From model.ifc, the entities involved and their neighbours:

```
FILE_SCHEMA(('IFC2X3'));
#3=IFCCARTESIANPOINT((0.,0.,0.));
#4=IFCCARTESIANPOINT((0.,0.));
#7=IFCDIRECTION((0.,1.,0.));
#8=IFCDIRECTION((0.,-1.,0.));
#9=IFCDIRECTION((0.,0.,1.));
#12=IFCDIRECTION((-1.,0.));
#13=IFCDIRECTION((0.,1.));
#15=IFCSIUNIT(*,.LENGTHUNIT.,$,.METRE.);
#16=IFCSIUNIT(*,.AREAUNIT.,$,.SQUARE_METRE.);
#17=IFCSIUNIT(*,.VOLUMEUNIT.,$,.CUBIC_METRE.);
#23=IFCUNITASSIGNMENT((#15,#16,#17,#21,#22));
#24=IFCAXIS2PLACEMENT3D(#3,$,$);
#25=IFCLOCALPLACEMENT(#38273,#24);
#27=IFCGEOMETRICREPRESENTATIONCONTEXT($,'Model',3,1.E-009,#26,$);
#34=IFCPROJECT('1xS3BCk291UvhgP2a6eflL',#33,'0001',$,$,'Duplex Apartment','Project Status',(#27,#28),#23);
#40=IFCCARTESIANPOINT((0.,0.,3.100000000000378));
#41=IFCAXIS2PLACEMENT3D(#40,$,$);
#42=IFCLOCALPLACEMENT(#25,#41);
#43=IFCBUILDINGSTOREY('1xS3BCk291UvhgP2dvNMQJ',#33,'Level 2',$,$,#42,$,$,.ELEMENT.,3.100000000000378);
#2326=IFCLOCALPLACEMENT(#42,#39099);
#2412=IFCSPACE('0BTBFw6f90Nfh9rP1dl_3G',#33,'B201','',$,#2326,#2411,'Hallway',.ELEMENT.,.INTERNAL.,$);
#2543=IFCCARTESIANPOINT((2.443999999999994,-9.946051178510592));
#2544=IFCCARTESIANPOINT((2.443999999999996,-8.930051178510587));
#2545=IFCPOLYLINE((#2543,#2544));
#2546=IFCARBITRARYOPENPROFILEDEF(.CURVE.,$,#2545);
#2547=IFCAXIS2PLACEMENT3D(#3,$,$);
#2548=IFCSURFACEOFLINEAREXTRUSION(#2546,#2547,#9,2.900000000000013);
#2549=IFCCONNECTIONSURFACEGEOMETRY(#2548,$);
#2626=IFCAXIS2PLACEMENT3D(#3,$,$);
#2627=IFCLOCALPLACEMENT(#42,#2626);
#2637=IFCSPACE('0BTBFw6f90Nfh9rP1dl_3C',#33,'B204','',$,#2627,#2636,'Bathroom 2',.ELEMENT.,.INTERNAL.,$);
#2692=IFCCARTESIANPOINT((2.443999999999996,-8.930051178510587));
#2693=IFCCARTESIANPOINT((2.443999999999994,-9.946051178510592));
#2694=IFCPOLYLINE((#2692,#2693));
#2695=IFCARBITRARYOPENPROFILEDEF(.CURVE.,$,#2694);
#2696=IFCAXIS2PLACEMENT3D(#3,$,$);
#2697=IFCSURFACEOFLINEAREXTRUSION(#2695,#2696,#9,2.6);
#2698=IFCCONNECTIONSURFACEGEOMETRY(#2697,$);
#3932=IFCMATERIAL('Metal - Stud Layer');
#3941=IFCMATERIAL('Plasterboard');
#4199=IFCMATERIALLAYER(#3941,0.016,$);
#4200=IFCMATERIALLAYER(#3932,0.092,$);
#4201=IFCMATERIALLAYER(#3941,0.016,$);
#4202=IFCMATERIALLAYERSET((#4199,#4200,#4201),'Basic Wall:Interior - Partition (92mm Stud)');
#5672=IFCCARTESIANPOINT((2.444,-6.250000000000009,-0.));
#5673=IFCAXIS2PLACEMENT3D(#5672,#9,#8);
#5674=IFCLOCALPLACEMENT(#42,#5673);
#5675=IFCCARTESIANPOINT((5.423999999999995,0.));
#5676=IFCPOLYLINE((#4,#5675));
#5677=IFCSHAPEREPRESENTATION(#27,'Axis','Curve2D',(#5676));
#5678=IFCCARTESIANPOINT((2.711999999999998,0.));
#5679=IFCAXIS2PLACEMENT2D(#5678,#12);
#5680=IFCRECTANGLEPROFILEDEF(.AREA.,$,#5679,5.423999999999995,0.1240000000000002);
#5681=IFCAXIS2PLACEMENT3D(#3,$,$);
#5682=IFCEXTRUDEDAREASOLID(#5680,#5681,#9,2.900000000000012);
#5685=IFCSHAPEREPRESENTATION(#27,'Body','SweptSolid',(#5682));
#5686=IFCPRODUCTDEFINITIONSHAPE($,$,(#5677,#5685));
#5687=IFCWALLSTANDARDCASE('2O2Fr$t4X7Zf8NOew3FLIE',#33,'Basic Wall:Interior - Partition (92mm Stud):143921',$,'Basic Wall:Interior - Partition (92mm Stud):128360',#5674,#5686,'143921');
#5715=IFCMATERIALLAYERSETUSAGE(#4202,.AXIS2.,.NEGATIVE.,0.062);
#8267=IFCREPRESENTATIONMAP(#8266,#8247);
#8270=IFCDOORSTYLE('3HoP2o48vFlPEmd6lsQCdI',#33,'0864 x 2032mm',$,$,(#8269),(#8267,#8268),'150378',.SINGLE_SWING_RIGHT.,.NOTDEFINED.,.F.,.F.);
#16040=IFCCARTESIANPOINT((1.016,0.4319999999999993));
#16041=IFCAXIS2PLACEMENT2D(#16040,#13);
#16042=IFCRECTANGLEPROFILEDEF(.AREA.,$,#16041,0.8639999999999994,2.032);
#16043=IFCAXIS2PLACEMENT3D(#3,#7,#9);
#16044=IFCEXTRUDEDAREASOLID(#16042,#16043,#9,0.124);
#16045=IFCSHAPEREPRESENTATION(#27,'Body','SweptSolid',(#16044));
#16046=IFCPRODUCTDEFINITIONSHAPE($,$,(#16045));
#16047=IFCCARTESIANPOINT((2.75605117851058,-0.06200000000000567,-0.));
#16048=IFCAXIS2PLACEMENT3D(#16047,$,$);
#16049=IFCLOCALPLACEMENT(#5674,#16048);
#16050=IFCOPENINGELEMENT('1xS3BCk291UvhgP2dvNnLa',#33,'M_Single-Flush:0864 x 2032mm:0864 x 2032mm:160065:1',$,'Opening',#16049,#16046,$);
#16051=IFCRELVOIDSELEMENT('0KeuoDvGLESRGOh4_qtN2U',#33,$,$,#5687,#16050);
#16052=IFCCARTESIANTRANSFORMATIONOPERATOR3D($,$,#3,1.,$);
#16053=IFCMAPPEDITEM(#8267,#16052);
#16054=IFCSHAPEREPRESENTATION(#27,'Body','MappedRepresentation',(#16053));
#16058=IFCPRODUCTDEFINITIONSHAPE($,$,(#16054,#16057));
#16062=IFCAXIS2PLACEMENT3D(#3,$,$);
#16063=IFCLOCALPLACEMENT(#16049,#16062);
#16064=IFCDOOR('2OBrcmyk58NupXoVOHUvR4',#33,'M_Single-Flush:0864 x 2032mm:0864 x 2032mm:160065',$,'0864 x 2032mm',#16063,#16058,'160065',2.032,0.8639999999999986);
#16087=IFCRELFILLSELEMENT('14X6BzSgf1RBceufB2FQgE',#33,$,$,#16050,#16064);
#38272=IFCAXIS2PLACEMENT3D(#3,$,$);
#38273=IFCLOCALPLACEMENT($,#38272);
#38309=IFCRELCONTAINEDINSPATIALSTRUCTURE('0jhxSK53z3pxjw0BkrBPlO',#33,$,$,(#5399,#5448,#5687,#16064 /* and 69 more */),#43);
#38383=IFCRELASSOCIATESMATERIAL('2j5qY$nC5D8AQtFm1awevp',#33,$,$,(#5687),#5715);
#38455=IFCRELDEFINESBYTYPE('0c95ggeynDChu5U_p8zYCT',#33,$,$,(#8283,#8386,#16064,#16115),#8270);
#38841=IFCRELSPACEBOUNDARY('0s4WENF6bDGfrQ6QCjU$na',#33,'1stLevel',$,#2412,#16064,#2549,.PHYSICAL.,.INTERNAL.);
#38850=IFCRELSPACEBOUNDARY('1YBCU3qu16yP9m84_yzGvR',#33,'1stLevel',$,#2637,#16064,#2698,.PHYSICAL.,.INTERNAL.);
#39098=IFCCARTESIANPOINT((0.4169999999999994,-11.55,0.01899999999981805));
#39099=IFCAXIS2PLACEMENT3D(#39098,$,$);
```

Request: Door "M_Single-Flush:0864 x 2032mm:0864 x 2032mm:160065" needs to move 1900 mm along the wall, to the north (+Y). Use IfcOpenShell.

```python
import numpy as np
import ifcopenshell
import ifcopenshell.api.geometry
import ifcopenshell.util.placement
import ifcopenshell.util.unit

model = ifcopenshell.open("model.ifc")
unit_scale = ifcopenshell.util.unit.calculate_unit_scale(model)

door = model.by_id(16064)
opening = door.FillsVoids[0].RelatingOpeningElement
wall = opening.VoidsElements[0].RelatingBuildingElement

wall_matrix = ifcopenshell.util.placement.get_local_placement(wall.ObjectPlacement)
shift = wall_matrix[:3, 0] * -1.9 / unit_scale
before = ifcopenshell.util.placement.get_local_placement(door.ObjectPlacement)[:3, 3].copy()

# The door is placed relative to its opening, so it follows when the opening moves.
matrix = ifcopenshell.util.placement.get_local_placement(opening.ObjectPlacement)
matrix[:3, 3] += shift
ifcopenshell.api.geometry.edit_object_placement(
    model, product=opening, matrix=matrix, is_si=False, should_transform_children=True
)

# Space boundary surfaces are stored in each space's coordinates; move them too.
for rel in door.ProvidesBoundaries:
    if not rel.ConnectionGeometry:
        continue
    surface = rel.ConnectionGeometry.SurfaceOnRelatingElement
    space_matrix = ifcopenshell.util.placement.get_local_placement(rel.RelatingSpace.ObjectPlacement)
    point = np.array(surface.Position.Location.Coordinates) + space_matrix[:3, :3].T @ shift
    surface.Position = model.createIfcAxis2Placement3D(
        model.createIfcCartesianPoint(point.tolist()), surface.Position.Axis, surface.Position.RefDirection
    )

after = ifcopenshell.util.placement.get_local_placement(door.ObjectPlacement)[:3, 3]
print("door moved by", (after - before).round(3) + 0.0)

model.write("model_rev.ifc")
```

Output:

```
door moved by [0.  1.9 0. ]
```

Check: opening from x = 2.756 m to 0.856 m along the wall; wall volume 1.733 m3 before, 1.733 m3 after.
